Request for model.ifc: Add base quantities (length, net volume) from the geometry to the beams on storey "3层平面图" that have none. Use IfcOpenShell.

First a look at what the model holds.

```python
import ifcopenshell
import ifcopenshell.util.element
import ifcopenshell.util.unit

model = ifcopenshell.open("model.ifc")
print(model.schema)
for unit_type in ("LENGTHUNIT", "AREAUNIT", "VOLUMEUNIT"):
    print(unit_type, ifcopenshell.util.unit.calculate_unit_scale(model, unit_type))
storey = next(s for s in model.by_type("IfcBuildingStorey") if s.Name == "3层平面图")
beams = [e for e in ifcopenshell.util.element.get_decomposition(storey) if e.is_a("IfcBeam")]
for e in sorted(beams, key=lambda e: e.id()):
    print(e.id(), e.is_a(), e.Name, list(ifcopenshell.util.element.get_psets(e, qtos_only=True)), sep=" | ")
```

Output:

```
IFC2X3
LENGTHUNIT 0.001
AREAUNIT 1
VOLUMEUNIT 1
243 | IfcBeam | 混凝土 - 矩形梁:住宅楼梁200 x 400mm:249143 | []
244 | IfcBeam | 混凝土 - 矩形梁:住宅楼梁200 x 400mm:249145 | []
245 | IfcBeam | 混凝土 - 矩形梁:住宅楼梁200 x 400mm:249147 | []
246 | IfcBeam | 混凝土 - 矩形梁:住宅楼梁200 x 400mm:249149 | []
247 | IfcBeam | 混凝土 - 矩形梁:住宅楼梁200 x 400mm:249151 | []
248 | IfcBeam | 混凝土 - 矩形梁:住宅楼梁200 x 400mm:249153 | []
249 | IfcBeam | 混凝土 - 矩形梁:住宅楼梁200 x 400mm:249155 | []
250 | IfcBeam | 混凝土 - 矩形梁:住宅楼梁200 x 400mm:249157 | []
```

```python
import ifcopenshell
import ifcopenshell.api.pset
import ifcopenshell.geom
import ifcopenshell.util.element
import ifcopenshell.util.shape
import ifcopenshell.util.unit

model = ifcopenshell.open("model.ifc")
unit_scale = ifcopenshell.util.unit.calculate_unit_scale(model)
volume_scale = ifcopenshell.util.unit.calculate_unit_scale(model, "VOLUMEUNIT")
settings = ifcopenshell.geom.settings()

storey = next(s for s in model.by_type("IfcBuildingStorey") if s.Name == "3层平面图")
beams = [e for e in ifcopenshell.util.element.get_decomposition(storey) if e.is_a("IfcBeam")]

for e in sorted(beams, key=lambda e: e.id()):
    if ifcopenshell.util.element.get_psets(e, qtos_only=True, should_inherit=False):
        continue
    # Geometry comes back in metres, in the element's own axes.
    shape = ifcopenshell.geom.create_shape(settings, e)
    values = {
        "Length": ifcopenshell.util.shape.get_max_xyz(shape.geometry) / unit_scale,
        "NetVolume": ifcopenshell.util.shape.get_volume(shape.geometry) / volume_scale,
    }
    qto = ifcopenshell.api.pset.add_qto(model, product=e, name="BaseQuantities")
    ifcopenshell.api.pset.edit_qto(model, qto=qto, properties=values)
    print(e.id(), {k: round(v, 3) for k, v in values.items()})

model.write("model_v2.ifc")
```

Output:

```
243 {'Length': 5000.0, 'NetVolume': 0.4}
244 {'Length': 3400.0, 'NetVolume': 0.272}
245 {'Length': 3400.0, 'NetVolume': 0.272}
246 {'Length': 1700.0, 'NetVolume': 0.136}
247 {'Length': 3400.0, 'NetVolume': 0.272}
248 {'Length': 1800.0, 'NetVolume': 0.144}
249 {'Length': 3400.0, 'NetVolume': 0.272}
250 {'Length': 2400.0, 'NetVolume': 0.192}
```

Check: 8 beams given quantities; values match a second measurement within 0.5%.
